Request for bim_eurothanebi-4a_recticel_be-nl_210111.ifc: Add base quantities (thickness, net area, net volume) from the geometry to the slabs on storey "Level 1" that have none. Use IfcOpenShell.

First a look at what the model holds.

```python
import ifcopenshell
import ifcopenshell.util.element
import ifcopenshell.util.unit

model = ifcopenshell.open("bim_eurothanebi-4a_recticel_be-nl_210111.ifc")
print(model.schema)
for unit_type in ("LENGTHUNIT", "AREAUNIT", "VOLUMEUNIT"):
    print(unit_type, ifcopenshell.util.unit.calculate_unit_scale(model, unit_type))
storey = next(s for s in model.by_type("IfcBuildingStorey") if s.Name == "Level 1")
slabs = [e for e in ifcopenshell.util.element.get_decomposition(storey) if e.is_a("IfcSlab")]
for e in sorted(slabs, key=lambda e: e.id()):
    print(e.id(), e.is_a(), e.Name, list(ifcopenshell.util.element.get_psets(e, qtos_only=True)), sep=" | ")
```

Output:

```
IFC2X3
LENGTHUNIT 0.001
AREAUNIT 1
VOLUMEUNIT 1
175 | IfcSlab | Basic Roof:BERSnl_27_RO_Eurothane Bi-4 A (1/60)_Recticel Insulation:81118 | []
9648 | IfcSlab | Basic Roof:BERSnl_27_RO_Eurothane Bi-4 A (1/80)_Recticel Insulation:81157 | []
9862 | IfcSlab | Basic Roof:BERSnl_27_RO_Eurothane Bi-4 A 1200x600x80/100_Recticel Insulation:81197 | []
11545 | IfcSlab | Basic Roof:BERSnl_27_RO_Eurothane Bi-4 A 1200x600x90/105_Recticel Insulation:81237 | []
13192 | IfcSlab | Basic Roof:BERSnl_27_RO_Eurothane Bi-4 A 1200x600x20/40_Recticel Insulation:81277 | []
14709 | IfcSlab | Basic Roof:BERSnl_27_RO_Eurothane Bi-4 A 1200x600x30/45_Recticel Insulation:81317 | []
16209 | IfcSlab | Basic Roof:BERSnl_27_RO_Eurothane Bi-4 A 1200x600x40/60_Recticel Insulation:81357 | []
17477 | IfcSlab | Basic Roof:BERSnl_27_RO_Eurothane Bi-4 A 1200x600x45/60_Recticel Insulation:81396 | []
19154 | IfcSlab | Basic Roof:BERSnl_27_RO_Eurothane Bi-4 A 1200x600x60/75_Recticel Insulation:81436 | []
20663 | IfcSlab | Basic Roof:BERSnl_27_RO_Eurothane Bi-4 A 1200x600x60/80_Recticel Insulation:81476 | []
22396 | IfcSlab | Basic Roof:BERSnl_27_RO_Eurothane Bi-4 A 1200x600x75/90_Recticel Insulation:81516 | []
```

```python
import ifcopenshell
import ifcopenshell.api.pset
import ifcopenshell.geom
import ifcopenshell.util.element
import ifcopenshell.util.shape
import ifcopenshell.util.unit

model = ifcopenshell.open("bim_eurothanebi-4a_recticel_be-nl_210111.ifc")
unit_scale = ifcopenshell.util.unit.calculate_unit_scale(model)
area_scale = ifcopenshell.util.unit.calculate_unit_scale(model, "AREAUNIT")
volume_scale = ifcopenshell.util.unit.calculate_unit_scale(model, "VOLUMEUNIT")
settings = ifcopenshell.geom.settings()

storey = next(s for s in model.by_type("IfcBuildingStorey") if s.Name == "Level 1")
slabs = [e for e in ifcopenshell.util.element.get_decomposition(storey) if e.is_a("IfcSlab")]

for e in sorted(slabs, key=lambda e: e.id()):
    if ifcopenshell.util.element.get_psets(e, qtos_only=True, should_inherit=False):
        continue
    # Geometry comes back in metres, in the element's own axes.
    shape = ifcopenshell.geom.create_shape(settings, e)
    values = {
        "Width": ifcopenshell.util.shape.get_z(shape.geometry) / unit_scale,
        "NetArea": ifcopenshell.util.shape.get_footprint_area(shape.geometry) / area_scale,
        "NetVolume": ifcopenshell.util.shape.get_volume(shape.geometry) / volume_scale,
    }
    qto = ifcopenshell.api.pset.add_qto(model, product=e, name="BaseQuantities")
    ifcopenshell.api.pset.edit_qto(model, qto=qto, properties=values)
    print(e.id(), {k: round(v, 3) for k, v in values.items()})

model.write("bim_eurothanebi-4a_recticel_be-nl_210111_v2.ifc")
```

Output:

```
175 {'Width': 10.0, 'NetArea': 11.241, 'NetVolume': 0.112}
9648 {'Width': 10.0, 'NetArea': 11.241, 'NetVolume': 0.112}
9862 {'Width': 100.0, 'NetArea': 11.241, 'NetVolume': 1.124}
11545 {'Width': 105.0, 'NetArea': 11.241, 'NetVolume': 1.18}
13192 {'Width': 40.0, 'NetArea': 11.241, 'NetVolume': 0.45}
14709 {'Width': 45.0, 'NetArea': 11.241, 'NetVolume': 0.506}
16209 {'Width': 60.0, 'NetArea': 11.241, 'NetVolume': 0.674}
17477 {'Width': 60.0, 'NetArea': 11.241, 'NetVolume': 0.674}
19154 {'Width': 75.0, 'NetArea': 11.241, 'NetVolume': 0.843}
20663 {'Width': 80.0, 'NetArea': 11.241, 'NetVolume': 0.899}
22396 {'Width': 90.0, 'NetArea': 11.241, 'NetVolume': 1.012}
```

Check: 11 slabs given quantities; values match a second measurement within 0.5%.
